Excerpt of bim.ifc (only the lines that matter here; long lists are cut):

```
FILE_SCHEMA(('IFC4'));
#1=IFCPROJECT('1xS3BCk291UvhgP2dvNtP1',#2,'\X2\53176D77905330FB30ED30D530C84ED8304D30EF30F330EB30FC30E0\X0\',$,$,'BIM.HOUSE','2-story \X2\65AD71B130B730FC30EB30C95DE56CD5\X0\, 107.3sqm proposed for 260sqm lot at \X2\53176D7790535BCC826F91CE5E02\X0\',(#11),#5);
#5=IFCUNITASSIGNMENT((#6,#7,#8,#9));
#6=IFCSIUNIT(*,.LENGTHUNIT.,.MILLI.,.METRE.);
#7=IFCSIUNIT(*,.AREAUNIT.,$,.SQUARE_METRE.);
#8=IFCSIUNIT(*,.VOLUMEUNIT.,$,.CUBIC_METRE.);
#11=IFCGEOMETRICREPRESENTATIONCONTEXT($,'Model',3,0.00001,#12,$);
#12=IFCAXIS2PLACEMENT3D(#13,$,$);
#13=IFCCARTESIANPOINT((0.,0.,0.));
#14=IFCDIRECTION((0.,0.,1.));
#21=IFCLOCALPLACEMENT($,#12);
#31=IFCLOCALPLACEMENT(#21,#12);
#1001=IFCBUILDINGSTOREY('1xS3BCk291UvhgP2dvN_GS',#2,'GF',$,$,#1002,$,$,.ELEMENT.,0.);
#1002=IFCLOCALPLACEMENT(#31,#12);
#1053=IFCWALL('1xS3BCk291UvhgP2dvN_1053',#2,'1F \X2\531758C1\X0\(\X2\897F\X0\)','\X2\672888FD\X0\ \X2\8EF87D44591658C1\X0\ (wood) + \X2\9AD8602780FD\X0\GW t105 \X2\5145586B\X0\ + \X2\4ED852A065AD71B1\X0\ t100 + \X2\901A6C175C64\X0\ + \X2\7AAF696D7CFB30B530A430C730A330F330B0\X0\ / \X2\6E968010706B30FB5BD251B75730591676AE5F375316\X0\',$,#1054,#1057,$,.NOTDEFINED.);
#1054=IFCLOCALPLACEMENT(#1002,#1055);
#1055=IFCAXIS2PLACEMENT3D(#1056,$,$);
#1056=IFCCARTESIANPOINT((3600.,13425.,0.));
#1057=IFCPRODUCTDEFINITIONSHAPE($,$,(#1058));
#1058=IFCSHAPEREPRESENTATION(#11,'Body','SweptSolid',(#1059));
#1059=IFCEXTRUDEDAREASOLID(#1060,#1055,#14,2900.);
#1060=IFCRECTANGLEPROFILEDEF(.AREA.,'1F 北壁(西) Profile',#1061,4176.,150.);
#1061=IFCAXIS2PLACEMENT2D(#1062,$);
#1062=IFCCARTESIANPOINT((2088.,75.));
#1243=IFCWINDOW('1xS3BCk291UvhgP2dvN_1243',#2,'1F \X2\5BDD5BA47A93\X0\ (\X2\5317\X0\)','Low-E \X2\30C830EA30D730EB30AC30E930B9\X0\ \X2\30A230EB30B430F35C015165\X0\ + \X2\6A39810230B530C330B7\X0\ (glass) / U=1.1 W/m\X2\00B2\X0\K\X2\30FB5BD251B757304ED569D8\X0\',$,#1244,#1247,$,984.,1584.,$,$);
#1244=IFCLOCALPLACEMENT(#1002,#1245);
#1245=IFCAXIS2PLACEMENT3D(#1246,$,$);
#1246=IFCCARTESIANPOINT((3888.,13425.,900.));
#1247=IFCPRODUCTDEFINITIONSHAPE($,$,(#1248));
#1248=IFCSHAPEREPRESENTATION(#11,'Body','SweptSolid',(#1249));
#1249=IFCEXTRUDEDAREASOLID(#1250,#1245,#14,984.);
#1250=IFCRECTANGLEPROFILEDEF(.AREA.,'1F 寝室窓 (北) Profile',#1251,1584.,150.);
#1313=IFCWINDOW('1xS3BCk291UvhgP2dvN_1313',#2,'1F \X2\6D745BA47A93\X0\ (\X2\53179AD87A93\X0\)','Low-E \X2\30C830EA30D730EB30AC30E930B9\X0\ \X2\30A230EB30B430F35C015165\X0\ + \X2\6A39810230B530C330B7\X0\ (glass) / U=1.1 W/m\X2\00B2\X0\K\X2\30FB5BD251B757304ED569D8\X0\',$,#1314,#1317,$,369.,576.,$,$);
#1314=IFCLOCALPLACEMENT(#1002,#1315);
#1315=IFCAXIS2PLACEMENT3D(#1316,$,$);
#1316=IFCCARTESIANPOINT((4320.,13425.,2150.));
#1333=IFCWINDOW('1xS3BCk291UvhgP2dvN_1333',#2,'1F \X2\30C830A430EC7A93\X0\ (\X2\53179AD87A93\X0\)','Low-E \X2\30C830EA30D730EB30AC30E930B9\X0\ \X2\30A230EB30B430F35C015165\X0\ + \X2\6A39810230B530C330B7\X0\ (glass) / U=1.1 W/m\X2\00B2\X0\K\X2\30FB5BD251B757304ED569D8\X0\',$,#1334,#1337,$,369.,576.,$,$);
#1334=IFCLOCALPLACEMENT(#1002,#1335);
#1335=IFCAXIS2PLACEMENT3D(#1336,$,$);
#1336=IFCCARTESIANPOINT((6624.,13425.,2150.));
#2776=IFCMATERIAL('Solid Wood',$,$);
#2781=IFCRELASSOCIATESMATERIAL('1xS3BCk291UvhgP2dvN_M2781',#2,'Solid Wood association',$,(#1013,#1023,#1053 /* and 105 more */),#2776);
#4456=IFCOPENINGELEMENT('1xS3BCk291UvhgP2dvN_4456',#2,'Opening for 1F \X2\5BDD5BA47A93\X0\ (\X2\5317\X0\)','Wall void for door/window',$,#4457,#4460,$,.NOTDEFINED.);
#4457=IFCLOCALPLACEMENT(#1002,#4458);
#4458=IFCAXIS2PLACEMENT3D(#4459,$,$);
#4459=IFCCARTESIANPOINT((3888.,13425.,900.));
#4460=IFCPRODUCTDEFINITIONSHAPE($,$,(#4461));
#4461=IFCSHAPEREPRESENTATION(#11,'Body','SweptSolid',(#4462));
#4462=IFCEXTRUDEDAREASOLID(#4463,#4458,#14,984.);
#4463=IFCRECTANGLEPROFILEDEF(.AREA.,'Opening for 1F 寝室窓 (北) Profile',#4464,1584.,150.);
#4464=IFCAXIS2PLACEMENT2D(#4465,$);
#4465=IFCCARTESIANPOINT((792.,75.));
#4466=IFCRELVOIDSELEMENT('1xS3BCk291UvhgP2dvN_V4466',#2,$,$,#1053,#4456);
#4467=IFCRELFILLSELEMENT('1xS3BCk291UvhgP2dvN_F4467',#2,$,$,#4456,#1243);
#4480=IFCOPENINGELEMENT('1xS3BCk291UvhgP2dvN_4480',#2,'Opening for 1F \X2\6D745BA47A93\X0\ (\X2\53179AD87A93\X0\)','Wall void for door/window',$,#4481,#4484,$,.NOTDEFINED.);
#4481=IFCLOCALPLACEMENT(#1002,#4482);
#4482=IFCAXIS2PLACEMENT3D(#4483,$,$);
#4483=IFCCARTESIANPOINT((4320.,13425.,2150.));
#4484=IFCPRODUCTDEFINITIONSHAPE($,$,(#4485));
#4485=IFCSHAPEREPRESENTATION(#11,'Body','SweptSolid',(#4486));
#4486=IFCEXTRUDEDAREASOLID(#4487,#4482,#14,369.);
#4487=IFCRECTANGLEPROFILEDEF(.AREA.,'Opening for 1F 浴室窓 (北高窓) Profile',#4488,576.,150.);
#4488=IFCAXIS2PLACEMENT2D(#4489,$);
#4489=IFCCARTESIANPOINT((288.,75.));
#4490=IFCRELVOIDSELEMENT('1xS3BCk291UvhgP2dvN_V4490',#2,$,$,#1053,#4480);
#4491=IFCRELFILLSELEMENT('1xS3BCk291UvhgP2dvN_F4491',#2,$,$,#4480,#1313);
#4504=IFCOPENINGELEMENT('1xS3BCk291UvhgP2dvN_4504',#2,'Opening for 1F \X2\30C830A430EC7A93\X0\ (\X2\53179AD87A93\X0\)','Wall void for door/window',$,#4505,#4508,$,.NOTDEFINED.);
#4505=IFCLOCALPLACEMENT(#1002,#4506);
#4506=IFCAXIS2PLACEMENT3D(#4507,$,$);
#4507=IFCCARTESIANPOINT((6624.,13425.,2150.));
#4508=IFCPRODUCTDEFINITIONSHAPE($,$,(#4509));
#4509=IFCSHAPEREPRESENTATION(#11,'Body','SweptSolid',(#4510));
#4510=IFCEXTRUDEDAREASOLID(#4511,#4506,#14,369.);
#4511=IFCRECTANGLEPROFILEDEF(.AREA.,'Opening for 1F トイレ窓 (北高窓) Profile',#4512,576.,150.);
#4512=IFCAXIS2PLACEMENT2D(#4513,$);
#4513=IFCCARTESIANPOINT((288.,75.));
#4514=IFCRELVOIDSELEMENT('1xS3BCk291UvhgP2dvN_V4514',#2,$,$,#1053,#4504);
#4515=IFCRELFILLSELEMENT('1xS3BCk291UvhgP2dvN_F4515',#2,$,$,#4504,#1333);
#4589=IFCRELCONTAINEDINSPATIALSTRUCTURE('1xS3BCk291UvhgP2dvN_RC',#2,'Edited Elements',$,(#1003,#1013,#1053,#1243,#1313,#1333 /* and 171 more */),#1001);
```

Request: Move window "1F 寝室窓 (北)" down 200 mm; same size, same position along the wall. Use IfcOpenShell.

```python
import numpy as np
import ifcopenshell
import ifcopenshell.api.geometry
import ifcopenshell.util.placement
import ifcopenshell.util.unit

model = ifcopenshell.open("bim.ifc")
unit_scale = ifcopenshell.util.unit.calculate_unit_scale(model)

window = model.by_guid("1xS3BCk291UvhgP2dvN_1243")
opening = window.FillsVoids[0].RelatingOpeningElement
dz = -200.0

shift = np.array([0.0, 0.0, dz])
# The window is not placed relative to its opening, so move both.
for product in (opening, window):
    matrix = ifcopenshell.util.placement.get_local_placement(product.ObjectPlacement)
    matrix[:3, 3] += shift
    ifcopenshell.api.geometry.edit_object_placement(model, product=product, matrix=matrix, is_si=False)

print(f"moved by {dz * unit_scale:+.3f} m")

model.write("bim_updated.ifc")
```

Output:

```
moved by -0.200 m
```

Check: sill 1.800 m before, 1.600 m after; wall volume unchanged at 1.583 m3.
